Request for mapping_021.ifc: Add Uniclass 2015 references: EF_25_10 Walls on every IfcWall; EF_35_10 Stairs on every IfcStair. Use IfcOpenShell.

First a look at what the model holds.

```python
import ifcopenshell

model = ifcopenshell.open("mapping_021.ifc")
print(model.schema)
print("classifications:", [c.Name for c in model.by_type("IfcClassification")])
for ifc_class in ("IfcDoor", "IfcRoof", "IfcStair", "IfcWall", "IfcWindow"):
    print(ifc_class, len(model.by_type(ifc_class)))
```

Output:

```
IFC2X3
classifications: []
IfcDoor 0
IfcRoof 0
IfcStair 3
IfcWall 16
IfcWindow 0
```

```python
import ifcopenshell
import ifcopenshell.api.classification

model = ifcopenshell.open("mapping_021.ifc")

# IFC2X3 requires Source and Edition and has no link from the project to the system.
system = model.create_entity("IfcClassification", Source="NBS", Edition="2015", Name="Uniclass 2015")

codes = {
    "IfcWall": ("EF_25_10", "Walls"),
    "IfcStair": ("EF_35_10", "Stairs"),
}
for ifc_class, (code, name) in codes.items():
    products = model.by_type(ifc_class)
    ifcopenshell.api.classification.add_reference(
        model, products=products, classification=system, identification=code, name=name
    )
    print(code, len(products))

model.write("mapping_021-out.ifc")
```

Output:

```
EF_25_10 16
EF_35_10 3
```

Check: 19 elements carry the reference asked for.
